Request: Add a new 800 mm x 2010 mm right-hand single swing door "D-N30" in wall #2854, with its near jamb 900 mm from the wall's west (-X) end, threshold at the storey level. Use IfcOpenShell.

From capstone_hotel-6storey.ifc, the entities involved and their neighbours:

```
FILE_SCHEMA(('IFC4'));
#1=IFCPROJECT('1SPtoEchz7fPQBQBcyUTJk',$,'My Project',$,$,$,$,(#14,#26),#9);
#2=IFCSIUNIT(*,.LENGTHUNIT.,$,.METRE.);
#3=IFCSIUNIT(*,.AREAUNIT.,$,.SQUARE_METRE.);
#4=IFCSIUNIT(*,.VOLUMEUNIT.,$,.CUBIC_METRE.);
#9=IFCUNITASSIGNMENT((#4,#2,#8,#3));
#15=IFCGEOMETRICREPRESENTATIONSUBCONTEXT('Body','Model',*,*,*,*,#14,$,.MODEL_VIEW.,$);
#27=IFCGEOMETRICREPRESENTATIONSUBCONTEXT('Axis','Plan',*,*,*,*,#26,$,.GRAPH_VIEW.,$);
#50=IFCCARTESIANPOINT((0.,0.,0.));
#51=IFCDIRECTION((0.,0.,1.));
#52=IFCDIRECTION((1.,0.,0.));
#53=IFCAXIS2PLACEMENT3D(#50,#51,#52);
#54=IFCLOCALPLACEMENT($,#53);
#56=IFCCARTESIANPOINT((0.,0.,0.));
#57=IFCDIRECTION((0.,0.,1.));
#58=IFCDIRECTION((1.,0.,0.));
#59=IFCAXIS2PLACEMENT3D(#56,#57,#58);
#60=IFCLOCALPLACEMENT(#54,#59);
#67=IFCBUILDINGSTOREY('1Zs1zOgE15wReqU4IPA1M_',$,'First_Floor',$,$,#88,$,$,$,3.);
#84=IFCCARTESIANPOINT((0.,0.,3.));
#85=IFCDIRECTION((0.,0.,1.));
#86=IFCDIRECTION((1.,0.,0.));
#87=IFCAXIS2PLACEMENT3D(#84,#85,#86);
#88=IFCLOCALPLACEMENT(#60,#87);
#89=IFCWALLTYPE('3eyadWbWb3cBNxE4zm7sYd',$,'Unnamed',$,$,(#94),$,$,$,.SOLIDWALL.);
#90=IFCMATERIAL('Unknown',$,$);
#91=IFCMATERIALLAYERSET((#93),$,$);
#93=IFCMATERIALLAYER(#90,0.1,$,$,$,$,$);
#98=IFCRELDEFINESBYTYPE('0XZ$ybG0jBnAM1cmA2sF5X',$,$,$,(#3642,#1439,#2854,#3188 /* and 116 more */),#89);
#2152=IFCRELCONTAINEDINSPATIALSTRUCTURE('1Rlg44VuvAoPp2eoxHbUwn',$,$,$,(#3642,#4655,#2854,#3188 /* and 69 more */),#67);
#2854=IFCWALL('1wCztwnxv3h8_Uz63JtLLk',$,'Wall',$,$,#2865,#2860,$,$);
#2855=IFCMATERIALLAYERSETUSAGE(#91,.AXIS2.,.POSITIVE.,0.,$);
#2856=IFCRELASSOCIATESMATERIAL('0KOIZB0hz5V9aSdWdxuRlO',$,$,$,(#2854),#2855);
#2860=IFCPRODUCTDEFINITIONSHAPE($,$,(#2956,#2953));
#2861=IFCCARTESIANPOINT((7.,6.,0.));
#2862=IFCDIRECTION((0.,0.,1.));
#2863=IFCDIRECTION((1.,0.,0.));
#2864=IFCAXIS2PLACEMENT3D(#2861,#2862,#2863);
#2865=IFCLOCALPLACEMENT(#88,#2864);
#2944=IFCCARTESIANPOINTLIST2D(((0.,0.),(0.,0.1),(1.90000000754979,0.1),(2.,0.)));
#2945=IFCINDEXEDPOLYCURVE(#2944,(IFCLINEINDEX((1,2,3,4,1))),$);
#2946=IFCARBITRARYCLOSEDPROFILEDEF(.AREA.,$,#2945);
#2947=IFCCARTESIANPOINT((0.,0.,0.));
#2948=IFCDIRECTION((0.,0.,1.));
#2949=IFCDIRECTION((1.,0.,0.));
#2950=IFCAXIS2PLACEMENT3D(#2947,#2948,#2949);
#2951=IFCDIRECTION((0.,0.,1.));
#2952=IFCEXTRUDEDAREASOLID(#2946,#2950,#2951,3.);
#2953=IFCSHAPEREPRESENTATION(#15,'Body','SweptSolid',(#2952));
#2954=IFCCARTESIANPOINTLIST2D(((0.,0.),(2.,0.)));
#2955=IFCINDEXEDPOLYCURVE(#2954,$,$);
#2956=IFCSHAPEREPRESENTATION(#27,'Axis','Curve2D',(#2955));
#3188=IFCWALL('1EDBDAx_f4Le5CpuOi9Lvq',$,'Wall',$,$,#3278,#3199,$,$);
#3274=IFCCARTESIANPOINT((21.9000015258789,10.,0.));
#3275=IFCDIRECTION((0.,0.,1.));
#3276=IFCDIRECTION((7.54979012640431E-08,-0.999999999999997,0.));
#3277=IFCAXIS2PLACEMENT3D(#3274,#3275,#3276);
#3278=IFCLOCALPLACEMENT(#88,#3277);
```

```python
import numpy as np
import ifcopenshell
import ifcopenshell.api.feature
import ifcopenshell.api.geometry
import ifcopenshell.api.root
import ifcopenshell.api.spatial
import ifcopenshell.geom
import ifcopenshell.util.element
import ifcopenshell.util.placement
import ifcopenshell.util.representation
import ifcopenshell.util.shape
import ifcopenshell.util.unit

model = ifcopenshell.open("capstone_hotel-6storey.ifc")
unit_scale = ifcopenshell.util.unit.calculate_unit_scale(model)
settings = ifcopenshell.geom.settings()


def volume(element):
    """Net volume in cubic metres, openings subtracted."""
    shape = ifcopenshell.geom.create_shape(settings, element)
    return ifcopenshell.util.shape.get_volume(shape.geometry)


wall = model.by_guid("1wCztwnxv3h8_Uz63JtLLk")
storey = ifcopenshell.util.element.get_container(wall, ifc_class="IfcBuildingStorey")
context = ifcopenshell.util.representation.get_context(model, "Model", "Body", "MODEL_VIEW")
before = volume(wall)

width, height, from_end, sill = 0.8, 2.01, 0.9, 0.0  # metres

# The wall runs along its own X axis, and the end named is its -X end.
wall_shape = ifcopenshell.geom.create_shape(settings, wall)
x, y, z = ifcopenshell.util.shape.get_vertices(wall_shape.geometry).T
start = x.min() + from_end
face, thickness = float(y.min()), float(y.max() - y.min())
wall_matrix = ifcopenshell.util.placement.get_local_placement(wall.ObjectPlacement)
level = ifcopenshell.util.placement.get_local_placement(storey.ObjectPlacement)[2, 3]


def in_wall(x, y):
    """Placement at x, y metres in the wall's axes, at sill height."""
    matrix = wall_matrix.copy()
    matrix[:, 3] = wall_matrix @ np.array([x / unit_scale, y / unit_scale, 0.0, 1.0])
    matrix[2, 3] = level + sill / unit_scale
    return matrix


# Opening: a box that overshoots both wall faces by 50 mm.
opening = ifcopenshell.api.root.create_entity(model, ifc_class="IfcOpeningElement", predefined_type="OPENING")
box = ifcopenshell.api.geometry.add_wall_representation(
    model, context=context, length=width, height=height, thickness=thickness + 0.1
)
ifcopenshell.api.geometry.assign_representation(model, product=opening, representation=box)
ifcopenshell.api.geometry.edit_object_placement(model, product=opening, matrix=in_wall(start, face - 0.05), is_si=False)
ifcopenshell.api.feature.add_feature(model, feature=opening, element=wall)

door = ifcopenshell.api.root.create_entity(model, ifc_class="IfcDoor", name="D-N30", predefined_type="DOOR")
door.OverallWidth, door.OverallHeight = width / unit_scale, height / unit_scale
door.OperationType = "SINGLE_SWING_RIGHT"
body = ifcopenshell.api.geometry.add_door_representation(
    model,
    context=context,
    overall_width=door.OverallWidth,
    overall_height=door.OverallHeight,
    operation_type="SINGLE_SWING_RIGHT",
    lining_properties={"LiningDepth": thickness / unit_scale, "ThresholdDepth": thickness / unit_scale},
)
ifcopenshell.api.geometry.assign_representation(model, product=door, representation=body)
ifcopenshell.api.spatial.assign_container(model, products=[door], relating_structure=storey)
ifcopenshell.api.feature.add_filling(model, opening=opening, element=door)

# The lining spans the wall, so the door starts at the wall face.
ifcopenshell.api.geometry.edit_object_placement(model, product=door, matrix=in_wall(start, face), is_si=False)

after = volume(wall)

print(f"wall volume {before:.3f} -> {after:.3f} m3")

model.write("capstone_hotel-6storey-out.ifc")
```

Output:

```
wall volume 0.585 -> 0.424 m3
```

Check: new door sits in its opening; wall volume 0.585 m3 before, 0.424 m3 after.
